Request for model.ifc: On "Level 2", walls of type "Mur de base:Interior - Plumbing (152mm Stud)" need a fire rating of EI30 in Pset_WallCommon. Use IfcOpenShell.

First a look at what the model holds.

```python
import ifcopenshell
import ifcopenshell.util.element

model = ifcopenshell.open("model.ifc")
print(model.schema)
storey = next(s for s in model.by_type("IfcBuildingStorey") if s.Name == "Level 2")
walls = [e for e in ifcopenshell.util.element.get_decomposition(storey) if e.is_a("IfcWall")]
seen = {}
for e in walls:
    element_type = ifcopenshell.util.element.get_type(e)
    key = (element_type.Name if element_type != e and element_type else None, ifcopenshell.util.element.get_pset(e, "Pset_WallCommon", "FireRating"))
    seen[key] = seen.get(key, 0) + 1
for (name, value), count in sorted(seen.items(), key=str):
    print(count, "x", name, "|", value)
```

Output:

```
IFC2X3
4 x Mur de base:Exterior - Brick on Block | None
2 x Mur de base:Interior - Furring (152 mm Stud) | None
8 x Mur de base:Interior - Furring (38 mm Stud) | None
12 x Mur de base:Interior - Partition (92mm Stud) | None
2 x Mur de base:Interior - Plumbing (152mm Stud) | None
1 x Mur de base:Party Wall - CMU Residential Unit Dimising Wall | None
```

```python
import ifcopenshell
import ifcopenshell.api.pset
import ifcopenshell.util.element

model = ifcopenshell.open("model.ifc")

storey = next(s for s in model.by_type("IfcBuildingStorey") if s.Name == "Level 2")
walls = [e for e in ifcopenshell.util.element.get_decomposition(storey) if e.is_a("IfcWall")]

count = 0
for e in walls:
    element_type = ifcopenshell.util.element.get_type(e)
    if element_type in (None, e) or element_type.Name != "Mur de base:Interior - Plumbing (152mm Stud)":
        continue
    # add_pset returns the element's existing set when there is one.
    pset = ifcopenshell.api.pset.add_pset(model, product=e, name="Pset_WallCommon")
    ifcopenshell.api.pset.edit_pset(model, pset=pset, properties={"FireRating": "EI30"})
    count += 1

print(count, "walls updated")

model.write("model_rev.ifc")
```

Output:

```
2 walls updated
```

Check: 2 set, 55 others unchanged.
